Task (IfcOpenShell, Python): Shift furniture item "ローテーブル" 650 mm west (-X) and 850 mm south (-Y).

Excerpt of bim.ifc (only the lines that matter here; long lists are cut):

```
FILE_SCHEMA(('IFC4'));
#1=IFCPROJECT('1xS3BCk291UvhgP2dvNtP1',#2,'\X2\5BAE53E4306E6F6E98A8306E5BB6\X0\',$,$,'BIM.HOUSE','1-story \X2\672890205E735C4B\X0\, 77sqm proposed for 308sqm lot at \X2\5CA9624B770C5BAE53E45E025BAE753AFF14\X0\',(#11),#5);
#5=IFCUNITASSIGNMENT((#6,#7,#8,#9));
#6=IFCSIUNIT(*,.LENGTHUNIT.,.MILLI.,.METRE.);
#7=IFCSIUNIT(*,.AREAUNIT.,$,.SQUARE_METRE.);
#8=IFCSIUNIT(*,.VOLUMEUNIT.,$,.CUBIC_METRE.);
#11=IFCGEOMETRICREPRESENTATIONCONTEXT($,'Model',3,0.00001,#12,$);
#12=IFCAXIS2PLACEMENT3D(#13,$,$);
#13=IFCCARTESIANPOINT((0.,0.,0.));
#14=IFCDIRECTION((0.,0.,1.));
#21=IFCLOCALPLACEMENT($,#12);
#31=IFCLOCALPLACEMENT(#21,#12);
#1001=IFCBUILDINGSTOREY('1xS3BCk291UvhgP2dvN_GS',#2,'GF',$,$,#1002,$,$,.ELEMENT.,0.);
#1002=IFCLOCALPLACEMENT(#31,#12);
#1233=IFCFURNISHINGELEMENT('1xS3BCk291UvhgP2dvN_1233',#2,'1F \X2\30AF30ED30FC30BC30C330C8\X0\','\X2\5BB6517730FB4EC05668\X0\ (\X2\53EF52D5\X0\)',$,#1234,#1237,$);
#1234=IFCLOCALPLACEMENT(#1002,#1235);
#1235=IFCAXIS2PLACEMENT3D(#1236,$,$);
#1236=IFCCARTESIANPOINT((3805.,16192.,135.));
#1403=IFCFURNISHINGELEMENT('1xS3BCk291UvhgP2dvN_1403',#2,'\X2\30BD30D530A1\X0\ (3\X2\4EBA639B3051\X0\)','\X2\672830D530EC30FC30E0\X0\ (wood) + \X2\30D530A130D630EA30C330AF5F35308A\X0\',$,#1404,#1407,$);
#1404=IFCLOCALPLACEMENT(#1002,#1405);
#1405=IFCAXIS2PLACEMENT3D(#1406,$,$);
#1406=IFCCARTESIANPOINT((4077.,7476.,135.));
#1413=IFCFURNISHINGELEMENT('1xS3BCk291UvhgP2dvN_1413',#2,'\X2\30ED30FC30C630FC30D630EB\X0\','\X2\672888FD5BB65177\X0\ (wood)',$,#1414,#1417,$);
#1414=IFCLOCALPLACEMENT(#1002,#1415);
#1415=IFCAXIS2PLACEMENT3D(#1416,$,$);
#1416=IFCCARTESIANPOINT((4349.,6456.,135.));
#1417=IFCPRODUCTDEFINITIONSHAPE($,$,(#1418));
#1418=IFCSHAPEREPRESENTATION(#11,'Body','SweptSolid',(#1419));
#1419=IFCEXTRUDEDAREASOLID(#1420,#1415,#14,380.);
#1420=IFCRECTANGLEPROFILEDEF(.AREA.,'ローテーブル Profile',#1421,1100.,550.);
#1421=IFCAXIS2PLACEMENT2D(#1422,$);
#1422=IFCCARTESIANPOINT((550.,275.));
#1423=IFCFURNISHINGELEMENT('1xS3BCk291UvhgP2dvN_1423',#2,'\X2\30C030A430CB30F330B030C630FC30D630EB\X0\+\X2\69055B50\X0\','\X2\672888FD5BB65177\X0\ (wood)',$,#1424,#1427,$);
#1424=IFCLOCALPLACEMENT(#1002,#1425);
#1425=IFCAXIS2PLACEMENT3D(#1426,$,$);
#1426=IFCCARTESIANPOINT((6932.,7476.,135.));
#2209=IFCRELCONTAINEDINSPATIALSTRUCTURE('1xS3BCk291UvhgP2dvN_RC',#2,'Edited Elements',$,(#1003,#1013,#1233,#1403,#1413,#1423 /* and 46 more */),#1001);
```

```python
import ifcopenshell
import ifcopenshell.api.geometry
import ifcopenshell.util.placement
import ifcopenshell.util.unit

model = ifcopenshell.open("bim.ifc")
unit_scale = ifcopenshell.util.unit.calculate_unit_scale(model)

item = model.by_guid("1xS3BCk291UvhgP2dvN_1413")
matrix = ifcopenshell.util.placement.get_local_placement(item.ObjectPlacement)
matrix[0, 3] -= 0.65 / unit_scale
matrix[1, 3] -= 0.85 / unit_scale
ifcopenshell.api.geometry.edit_object_placement(model, product=item, matrix=matrix, is_si=False)

print(ifcopenshell.util.placement.get_local_placement(item.ObjectPlacement).round(3) + 0.0)

model.write("bim_v2.ifc")
```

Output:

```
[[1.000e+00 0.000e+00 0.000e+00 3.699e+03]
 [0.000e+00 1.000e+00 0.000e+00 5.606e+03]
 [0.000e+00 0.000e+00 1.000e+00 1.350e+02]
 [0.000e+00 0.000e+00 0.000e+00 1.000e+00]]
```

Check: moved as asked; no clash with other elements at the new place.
